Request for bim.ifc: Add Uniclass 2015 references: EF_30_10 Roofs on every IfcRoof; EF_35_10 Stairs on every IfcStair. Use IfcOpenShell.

First a look at what the model holds.

```python
import ifcopenshell

model = ifcopenshell.open("bim.ifc")
print(model.schema)
print("classifications:", [c.Name for c in model.by_type("IfcClassification")])
for ifc_class in ("IfcDoor", "IfcRoof", "IfcStair", "IfcWall", "IfcWindow"):
    print(ifc_class, len(model.by_type(ifc_class)))
```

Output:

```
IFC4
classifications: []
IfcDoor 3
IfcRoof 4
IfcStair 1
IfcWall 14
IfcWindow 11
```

```python
import ifcopenshell
import ifcopenshell.api.classification

model = ifcopenshell.open("bim.ifc")

system = ifcopenshell.api.classification.add_classification(model, classification="Uniclass 2015")

codes = {
    "IfcRoof": ("EF_30_10", "Roofs"),
    "IfcStair": ("EF_35_10", "Stairs"),
}
for ifc_class, (code, name) in codes.items():
    products = model.by_type(ifc_class)
    ifcopenshell.api.classification.add_reference(
        model, products=products, classification=system, identification=code, name=name
    )
    print(code, len(products))

model.write("bim-out.ifc")
```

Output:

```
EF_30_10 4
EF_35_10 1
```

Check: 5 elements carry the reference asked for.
